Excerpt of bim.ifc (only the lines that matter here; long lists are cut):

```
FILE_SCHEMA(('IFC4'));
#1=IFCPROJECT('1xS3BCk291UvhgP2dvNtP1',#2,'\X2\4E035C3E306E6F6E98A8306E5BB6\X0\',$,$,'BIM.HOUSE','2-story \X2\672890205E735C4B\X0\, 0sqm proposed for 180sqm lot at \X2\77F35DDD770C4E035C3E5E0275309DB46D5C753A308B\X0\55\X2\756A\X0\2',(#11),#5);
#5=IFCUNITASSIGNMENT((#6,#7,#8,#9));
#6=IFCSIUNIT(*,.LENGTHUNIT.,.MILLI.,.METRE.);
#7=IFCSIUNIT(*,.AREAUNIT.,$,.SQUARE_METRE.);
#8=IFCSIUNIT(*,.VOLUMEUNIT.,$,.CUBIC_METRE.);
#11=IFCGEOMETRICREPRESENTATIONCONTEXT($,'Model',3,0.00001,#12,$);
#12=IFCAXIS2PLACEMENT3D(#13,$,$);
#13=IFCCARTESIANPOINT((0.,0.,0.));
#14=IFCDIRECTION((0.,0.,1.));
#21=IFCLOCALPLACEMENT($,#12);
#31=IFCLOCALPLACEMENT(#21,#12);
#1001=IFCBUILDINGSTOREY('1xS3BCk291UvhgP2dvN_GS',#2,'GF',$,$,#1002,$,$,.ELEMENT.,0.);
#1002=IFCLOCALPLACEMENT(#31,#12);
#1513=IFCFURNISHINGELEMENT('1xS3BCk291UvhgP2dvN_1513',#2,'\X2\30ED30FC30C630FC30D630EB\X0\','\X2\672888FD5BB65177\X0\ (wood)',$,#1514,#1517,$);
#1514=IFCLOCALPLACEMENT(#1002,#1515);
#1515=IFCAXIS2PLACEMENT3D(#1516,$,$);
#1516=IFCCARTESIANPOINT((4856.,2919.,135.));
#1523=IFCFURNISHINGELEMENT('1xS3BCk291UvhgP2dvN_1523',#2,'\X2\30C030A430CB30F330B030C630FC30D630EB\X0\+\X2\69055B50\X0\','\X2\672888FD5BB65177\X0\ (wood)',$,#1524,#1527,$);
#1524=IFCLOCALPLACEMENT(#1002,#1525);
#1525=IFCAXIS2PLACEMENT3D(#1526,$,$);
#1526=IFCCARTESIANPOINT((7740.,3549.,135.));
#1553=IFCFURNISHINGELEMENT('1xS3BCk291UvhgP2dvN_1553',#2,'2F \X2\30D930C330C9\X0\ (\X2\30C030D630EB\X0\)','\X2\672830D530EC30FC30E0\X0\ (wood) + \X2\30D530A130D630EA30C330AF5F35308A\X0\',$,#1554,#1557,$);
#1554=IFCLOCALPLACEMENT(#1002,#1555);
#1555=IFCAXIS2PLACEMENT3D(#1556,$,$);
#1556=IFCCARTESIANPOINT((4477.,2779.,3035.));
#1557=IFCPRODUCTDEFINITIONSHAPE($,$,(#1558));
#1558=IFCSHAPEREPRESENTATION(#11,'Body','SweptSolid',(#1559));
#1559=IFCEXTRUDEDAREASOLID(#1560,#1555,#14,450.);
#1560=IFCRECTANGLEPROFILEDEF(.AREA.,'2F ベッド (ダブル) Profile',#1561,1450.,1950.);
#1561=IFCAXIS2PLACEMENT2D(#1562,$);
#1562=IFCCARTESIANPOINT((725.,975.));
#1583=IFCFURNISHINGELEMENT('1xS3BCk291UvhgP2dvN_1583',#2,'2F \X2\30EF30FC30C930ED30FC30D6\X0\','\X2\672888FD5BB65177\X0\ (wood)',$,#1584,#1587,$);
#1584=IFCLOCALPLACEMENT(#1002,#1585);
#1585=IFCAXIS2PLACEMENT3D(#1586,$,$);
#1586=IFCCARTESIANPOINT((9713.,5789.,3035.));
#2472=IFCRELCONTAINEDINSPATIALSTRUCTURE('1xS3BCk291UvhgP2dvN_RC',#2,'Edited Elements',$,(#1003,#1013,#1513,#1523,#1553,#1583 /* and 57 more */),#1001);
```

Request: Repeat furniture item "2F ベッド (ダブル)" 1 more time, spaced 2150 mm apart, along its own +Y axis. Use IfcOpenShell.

```python
import ifcopenshell
import ifcopenshell.api.geometry
import ifcopenshell.api.root
import ifcopenshell.util.element
import ifcopenshell.util.placement
import ifcopenshell.util.unit

model = ifcopenshell.open("bim.ifc")
unit_scale = ifcopenshell.util.unit.calculate_unit_scale(model)


def reuse_history(source, copy):
    """copy_class also copies each property set's owner history, people and application; keep the originals."""
    for rel in copy.IsDefinedBy:
        if rel.is_a("IfcRelDefinesByProperties") and (history := rel.RelatingPropertyDefinition.OwnerHistory):
            rel.RelatingPropertyDefinition.OwnerHistory = source.OwnerHistory
            ifcopenshell.util.element.remove_deep2(model, history)


source = model.by_guid("1xS3BCk291UvhgP2dvN_1553")
base = ifcopenshell.util.placement.get_local_placement(source.ObjectPlacement)
step = base[:3, 1] * 2.15 / unit_scale

for i in range(1, 2):
    copy = ifcopenshell.api.root.copy_class(model, product=source)
    copy.Representation = ifcopenshell.util.element.copy_deep(
        model, source.Representation, exclude=["IfcGeometricRepresentationContext", "IfcRepresentationMap"]
    )
    reuse_history(source, copy)
    matrix = base.copy()
    matrix[:3, 3] += i * step
    print("added at", matrix[:3, 3].round(3) + 0.0)
    ifcopenshell.api.geometry.edit_object_placement(model, product=copy, matrix=matrix, is_si=False)

model.write("bim-out.ifc")
```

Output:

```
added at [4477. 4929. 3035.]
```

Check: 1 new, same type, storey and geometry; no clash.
